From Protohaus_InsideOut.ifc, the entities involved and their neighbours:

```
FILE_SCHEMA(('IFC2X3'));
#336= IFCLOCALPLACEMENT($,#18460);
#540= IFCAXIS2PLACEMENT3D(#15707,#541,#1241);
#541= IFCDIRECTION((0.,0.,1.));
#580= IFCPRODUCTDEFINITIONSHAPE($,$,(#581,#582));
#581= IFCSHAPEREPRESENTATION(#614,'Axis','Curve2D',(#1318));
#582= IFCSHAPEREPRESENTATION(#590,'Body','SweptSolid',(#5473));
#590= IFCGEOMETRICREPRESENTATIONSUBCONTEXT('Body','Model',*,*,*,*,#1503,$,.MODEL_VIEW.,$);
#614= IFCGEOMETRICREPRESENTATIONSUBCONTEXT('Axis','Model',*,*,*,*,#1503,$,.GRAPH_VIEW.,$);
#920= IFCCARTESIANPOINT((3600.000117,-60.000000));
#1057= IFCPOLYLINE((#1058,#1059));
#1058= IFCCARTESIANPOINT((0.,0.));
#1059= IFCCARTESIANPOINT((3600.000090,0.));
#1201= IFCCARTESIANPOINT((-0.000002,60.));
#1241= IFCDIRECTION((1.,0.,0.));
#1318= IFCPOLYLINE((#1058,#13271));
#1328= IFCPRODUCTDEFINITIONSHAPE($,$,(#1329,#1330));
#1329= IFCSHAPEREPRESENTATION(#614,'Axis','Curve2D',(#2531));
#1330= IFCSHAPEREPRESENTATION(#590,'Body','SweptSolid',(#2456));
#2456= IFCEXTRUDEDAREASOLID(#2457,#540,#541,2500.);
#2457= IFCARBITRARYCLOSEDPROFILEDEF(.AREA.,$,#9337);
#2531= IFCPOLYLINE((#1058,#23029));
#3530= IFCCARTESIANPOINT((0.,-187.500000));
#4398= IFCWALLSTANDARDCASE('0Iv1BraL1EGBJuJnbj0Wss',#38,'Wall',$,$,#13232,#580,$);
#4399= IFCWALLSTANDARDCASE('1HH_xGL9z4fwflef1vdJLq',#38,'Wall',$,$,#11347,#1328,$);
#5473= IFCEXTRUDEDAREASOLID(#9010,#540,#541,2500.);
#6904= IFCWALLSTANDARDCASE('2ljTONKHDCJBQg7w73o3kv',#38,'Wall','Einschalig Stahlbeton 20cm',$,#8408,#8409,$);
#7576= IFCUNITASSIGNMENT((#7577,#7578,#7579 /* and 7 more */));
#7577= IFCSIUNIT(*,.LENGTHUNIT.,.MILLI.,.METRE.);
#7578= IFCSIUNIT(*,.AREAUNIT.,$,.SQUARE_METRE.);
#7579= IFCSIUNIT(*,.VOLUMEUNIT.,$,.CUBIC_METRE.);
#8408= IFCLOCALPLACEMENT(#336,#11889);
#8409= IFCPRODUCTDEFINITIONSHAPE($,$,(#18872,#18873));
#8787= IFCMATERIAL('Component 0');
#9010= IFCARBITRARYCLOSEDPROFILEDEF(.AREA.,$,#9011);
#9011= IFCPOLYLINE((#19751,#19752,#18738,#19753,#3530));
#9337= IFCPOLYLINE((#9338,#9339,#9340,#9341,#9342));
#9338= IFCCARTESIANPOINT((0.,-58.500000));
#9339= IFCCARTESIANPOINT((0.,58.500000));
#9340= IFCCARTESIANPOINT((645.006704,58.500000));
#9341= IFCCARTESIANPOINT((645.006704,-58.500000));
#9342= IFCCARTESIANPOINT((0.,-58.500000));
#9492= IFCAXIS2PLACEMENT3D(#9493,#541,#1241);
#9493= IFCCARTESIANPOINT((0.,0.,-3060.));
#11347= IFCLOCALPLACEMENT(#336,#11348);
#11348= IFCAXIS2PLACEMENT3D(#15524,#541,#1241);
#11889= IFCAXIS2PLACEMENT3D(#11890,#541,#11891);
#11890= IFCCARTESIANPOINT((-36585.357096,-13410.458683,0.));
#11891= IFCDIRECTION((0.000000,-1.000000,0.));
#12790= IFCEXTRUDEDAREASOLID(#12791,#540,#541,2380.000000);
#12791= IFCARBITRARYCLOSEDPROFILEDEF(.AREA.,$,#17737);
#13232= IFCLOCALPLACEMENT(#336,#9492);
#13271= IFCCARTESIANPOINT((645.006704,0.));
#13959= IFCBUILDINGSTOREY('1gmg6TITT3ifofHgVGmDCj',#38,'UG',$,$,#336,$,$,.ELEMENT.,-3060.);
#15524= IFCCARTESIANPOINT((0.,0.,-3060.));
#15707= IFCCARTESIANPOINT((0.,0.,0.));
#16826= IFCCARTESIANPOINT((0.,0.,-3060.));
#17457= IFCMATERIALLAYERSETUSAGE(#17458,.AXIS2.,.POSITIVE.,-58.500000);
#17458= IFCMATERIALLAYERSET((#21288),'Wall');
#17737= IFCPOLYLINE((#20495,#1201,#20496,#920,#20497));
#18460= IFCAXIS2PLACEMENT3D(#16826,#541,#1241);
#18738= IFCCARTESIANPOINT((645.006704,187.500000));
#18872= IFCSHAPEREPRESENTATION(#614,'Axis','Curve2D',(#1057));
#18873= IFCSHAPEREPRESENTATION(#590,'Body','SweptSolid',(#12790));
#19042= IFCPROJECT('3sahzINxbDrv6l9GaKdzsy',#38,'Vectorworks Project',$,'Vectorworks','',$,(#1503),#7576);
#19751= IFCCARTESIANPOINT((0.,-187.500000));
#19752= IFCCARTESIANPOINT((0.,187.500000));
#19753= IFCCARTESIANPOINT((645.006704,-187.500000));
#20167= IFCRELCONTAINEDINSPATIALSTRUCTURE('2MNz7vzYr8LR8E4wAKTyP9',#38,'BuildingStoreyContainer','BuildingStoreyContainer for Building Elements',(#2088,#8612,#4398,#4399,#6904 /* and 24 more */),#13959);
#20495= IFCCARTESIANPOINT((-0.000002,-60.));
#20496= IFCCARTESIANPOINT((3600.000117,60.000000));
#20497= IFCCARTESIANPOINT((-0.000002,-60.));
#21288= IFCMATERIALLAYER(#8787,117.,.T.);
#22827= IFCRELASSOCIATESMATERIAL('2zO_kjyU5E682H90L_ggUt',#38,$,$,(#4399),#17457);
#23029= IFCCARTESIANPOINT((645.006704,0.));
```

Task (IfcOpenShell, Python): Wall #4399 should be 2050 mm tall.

```python
import ifcopenshell
import ifcopenshell.geom
import ifcopenshell.util.representation
import ifcopenshell.util.shape
import ifcopenshell.util.unit

model = ifcopenshell.open("Protohaus_InsideOut.ifc")
unit_scale = ifcopenshell.util.unit.calculate_unit_scale(model)
settings = ifcopenshell.geom.settings()


def volume(element):
    """Net volume in cubic metres, openings subtracted."""
    shape = ifcopenshell.geom.create_shape(settings, element)
    return ifcopenshell.util.shape.get_volume(shape.geometry)


wall = model.by_guid("1HH_xGL9z4fwflef1vdJLq")
before = volume(wall)

body = ifcopenshell.util.representation.get_representation(wall, "Model", "Body")
solid = body.Items[0]
old_height = solid.Depth
solid.Depth = 2.05 / unit_scale
after = volume(wall)

print(f"height {old_height:g} -> {solid.Depth:g}, volume {before:.3f} -> {after:.3f} m3")

model.write("Protohaus_InsideOut-out.ifc")
```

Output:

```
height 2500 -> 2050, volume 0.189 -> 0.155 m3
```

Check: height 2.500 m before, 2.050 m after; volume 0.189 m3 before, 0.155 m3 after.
